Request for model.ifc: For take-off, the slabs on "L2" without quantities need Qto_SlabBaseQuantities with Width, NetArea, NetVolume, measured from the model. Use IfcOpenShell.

First a look at what the model holds.

```python
import ifcopenshell
import ifcopenshell.util.element
import ifcopenshell.util.unit

model = ifcopenshell.open("model.ifc")
print(model.schema)
for unit_type in ("LENGTHUNIT", "AREAUNIT", "VOLUMEUNIT"):
    print(unit_type, ifcopenshell.util.unit.calculate_unit_scale(model, unit_type))
storey = next(s for s in model.by_type("IfcBuildingStorey") if s.Name == "L2")
slabs = [e for e in ifcopenshell.util.element.get_decomposition(storey) if e.is_a("IfcSlab")]
for e in sorted(slabs, key=lambda e: e.id()):
    print(e.id(), e.is_a(), e.Name, list(ifcopenshell.util.element.get_psets(e, qtos_only=True)), sep=" | ")
```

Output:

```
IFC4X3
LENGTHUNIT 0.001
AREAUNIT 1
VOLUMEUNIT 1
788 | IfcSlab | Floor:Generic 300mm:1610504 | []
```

```python
import ifcopenshell
import ifcopenshell.api.pset
import ifcopenshell.geom
import ifcopenshell.util.element
import ifcopenshell.util.shape
import ifcopenshell.util.unit

model = ifcopenshell.open("model.ifc")
unit_scale = ifcopenshell.util.unit.calculate_unit_scale(model)
area_scale = ifcopenshell.util.unit.calculate_unit_scale(model, "AREAUNIT")
volume_scale = ifcopenshell.util.unit.calculate_unit_scale(model, "VOLUMEUNIT")
settings = ifcopenshell.geom.settings()

storey = next(s for s in model.by_type("IfcBuildingStorey") if s.Name == "L2")
slabs = [e for e in ifcopenshell.util.element.get_decomposition(storey) if e.is_a("IfcSlab")]

for e in sorted(slabs, key=lambda e: e.id()):
    if ifcopenshell.util.element.get_psets(e, qtos_only=True, should_inherit=False):
        continue
    # Geometry comes back in metres, in the element's own axes.
    shape = ifcopenshell.geom.create_shape(settings, e)
    values = {
        "Width": ifcopenshell.util.shape.get_z(shape.geometry) / unit_scale,
        "NetArea": ifcopenshell.util.shape.get_footprint_area(shape.geometry) / area_scale,
        "NetVolume": ifcopenshell.util.shape.get_volume(shape.geometry) / volume_scale,
    }
    qto = ifcopenshell.api.pset.add_qto(model, product=e, name="Qto_SlabBaseQuantities")
    ifcopenshell.api.pset.edit_qto(model, qto=qto, properties=values)
    print(e.id(), {k: round(v, 3) for k, v in values.items()})

model.write("model_rev.ifc")
```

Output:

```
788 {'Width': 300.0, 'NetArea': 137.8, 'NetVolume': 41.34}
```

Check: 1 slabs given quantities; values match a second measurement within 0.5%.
